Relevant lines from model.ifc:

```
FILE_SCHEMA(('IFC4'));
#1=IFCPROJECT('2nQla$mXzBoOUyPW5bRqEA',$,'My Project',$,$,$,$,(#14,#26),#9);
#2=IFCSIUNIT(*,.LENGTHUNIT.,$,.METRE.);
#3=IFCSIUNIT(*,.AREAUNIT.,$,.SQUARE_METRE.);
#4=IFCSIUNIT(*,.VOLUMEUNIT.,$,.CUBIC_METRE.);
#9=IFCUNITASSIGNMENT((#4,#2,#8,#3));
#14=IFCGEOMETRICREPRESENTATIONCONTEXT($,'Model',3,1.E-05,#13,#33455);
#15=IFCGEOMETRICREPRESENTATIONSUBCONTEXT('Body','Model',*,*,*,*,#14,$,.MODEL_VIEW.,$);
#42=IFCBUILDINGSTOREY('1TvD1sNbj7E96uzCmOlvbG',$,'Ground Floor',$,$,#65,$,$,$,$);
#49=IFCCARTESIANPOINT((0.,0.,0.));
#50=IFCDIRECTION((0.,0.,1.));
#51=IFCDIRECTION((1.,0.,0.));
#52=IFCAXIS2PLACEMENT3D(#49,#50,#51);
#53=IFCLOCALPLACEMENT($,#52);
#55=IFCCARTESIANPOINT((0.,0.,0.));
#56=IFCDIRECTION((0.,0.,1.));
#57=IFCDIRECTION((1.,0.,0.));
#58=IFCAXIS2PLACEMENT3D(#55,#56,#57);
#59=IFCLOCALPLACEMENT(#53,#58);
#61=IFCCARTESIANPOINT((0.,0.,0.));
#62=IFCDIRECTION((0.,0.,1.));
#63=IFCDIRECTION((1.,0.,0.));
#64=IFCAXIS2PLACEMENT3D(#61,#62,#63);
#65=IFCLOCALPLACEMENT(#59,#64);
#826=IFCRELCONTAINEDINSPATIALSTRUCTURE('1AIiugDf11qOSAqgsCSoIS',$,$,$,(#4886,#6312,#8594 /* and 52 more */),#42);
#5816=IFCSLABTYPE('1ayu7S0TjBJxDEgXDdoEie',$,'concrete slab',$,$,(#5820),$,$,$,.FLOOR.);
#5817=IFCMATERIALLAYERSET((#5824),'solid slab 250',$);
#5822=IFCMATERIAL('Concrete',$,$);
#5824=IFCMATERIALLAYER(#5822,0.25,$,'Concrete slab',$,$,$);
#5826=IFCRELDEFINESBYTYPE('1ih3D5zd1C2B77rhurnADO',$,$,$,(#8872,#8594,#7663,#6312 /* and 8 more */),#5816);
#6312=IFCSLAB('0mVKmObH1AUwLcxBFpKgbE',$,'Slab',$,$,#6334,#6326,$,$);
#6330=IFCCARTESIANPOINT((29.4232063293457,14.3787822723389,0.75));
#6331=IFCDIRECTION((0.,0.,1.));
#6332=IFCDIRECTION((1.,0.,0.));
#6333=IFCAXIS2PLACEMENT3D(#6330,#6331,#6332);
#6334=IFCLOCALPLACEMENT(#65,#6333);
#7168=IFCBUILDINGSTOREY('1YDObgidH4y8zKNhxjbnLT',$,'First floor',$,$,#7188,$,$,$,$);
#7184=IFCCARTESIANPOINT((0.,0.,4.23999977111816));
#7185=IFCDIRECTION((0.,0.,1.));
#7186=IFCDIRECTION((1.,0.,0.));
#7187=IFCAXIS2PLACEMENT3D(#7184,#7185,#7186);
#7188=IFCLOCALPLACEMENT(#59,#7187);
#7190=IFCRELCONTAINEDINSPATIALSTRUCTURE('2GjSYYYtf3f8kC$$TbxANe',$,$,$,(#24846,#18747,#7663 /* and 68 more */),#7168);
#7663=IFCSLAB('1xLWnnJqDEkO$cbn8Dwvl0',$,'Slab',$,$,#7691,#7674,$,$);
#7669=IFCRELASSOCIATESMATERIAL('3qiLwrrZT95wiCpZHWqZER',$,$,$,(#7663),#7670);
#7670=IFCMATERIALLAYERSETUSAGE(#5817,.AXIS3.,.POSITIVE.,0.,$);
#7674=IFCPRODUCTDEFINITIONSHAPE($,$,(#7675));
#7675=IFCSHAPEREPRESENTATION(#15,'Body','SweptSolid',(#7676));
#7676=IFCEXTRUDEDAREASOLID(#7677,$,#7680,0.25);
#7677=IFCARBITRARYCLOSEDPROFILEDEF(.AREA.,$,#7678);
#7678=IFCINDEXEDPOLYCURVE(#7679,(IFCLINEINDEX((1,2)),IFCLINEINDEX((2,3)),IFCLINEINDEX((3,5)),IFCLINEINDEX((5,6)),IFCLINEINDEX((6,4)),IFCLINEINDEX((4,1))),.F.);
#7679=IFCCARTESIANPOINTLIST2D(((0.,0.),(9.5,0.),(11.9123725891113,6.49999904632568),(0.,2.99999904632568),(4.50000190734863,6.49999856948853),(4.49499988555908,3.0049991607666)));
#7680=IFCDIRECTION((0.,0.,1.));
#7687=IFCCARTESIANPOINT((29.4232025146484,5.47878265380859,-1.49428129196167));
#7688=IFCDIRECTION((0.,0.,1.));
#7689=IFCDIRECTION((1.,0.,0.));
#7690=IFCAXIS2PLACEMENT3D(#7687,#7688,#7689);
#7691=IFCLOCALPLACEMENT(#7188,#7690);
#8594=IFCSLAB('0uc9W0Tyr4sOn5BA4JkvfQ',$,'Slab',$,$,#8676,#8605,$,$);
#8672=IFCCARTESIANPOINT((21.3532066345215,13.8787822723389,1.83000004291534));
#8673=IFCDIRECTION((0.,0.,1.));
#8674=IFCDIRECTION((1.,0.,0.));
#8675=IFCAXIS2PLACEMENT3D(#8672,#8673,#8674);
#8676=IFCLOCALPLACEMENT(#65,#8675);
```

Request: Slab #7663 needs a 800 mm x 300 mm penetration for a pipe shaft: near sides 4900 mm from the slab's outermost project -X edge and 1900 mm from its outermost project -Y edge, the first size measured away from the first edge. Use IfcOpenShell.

```python
import numpy as np
import ifcopenshell
import ifcopenshell.api.feature
import ifcopenshell.api.geometry
import ifcopenshell.api.root
import ifcopenshell.geom
import ifcopenshell.util.placement
import ifcopenshell.util.representation
import ifcopenshell.util.shape
import ifcopenshell.util.unit

model = ifcopenshell.open("model.ifc")
unit_scale = ifcopenshell.util.unit.calculate_unit_scale(model)
settings = ifcopenshell.geom.settings()


def volume(element):
    """Net volume in cubic metres, openings subtracted."""
    shape = ifcopenshell.geom.create_shape(settings, element)
    return ifcopenshell.util.shape.get_volume(shape.geometry)


slab = model.by_guid("1xLWnnJqDEkO$cbn8Dwvl0")
before = volume(slab)

# Extent in the slab's own axes, in metres. The edges named are its -X and -Y sides.
slab_shape = ifcopenshell.geom.create_shape(settings, slab)
vertices = ifcopenshell.util.shape.get_vertices(slab_shape.geometry)
x_min, y_min, bottom = vertices.min(axis=0)
top = vertices[:, 2].max()

opening = ifcopenshell.api.root.create_entity(model, ifc_class="IfcOpeningElement", name="Pipe shaft opening", predefined_type="OPENING")
context = ifcopenshell.util.representation.get_context(model, "Model", "Body", "MODEL_VIEW")
width, depth = 0.8, 0.3
outline = [(0.0, 0.0), (width, 0.0), (width, depth), (0.0, depth), (0.0, 0.0)]
# Overshoot both faces by 50 mm so the cut is clean.
shape = ifcopenshell.api.geometry.add_slab_representation(
    model, context=context, depth=top - bottom + 0.1, polyline=outline
)
ifcopenshell.api.geometry.assign_representation(model, product=opening, representation=shape)

matrix = ifcopenshell.util.placement.get_local_placement(slab.ObjectPlacement)
matrix[:, 3] = matrix @ np.append(np.array([x_min + 4.9, y_min + 1.9, bottom - 0.05]) / unit_scale, 1.0)
ifcopenshell.api.geometry.edit_object_placement(model, product=opening, matrix=matrix, is_si=False)
ifcopenshell.api.feature.add_feature(model, feature=opening, element=slab)

after = volume(slab)

print(f"slab volume {before:.3f} -> {after:.3f} m3")

model.write("model_updated.ifc")
```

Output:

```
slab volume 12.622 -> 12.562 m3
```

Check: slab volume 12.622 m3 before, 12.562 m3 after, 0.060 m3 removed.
